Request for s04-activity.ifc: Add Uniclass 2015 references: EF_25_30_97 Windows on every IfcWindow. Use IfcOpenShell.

First a look at what the model holds.

```python
import ifcopenshell

model = ifcopenshell.open("s04-activity.ifc")
print(model.schema)
print("classifications:", [c.Name for c in model.by_type("IfcClassification")])
for ifc_class in ("IfcDoor", "IfcRoof", "IfcStair", "IfcWall", "IfcWindow"):
    print(ifc_class, len(model.by_type(ifc_class)))
```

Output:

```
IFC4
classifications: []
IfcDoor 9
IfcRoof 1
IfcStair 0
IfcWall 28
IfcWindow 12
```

```python
import ifcopenshell
import ifcopenshell.api.classification

model = ifcopenshell.open("s04-activity.ifc")

system = ifcopenshell.api.classification.add_classification(model, classification="Uniclass 2015")

codes = {
    "IfcWindow": ("EF_25_30_97", "Windows"),
}
for ifc_class, (code, name) in codes.items():
    products = model.by_type(ifc_class)
    ifcopenshell.api.classification.add_reference(
        model, products=products, classification=system, identification=code, name=name
    )
    print(code, len(products))

model.write("s04-activity_v2.ifc")
```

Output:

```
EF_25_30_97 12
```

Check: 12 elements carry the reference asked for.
